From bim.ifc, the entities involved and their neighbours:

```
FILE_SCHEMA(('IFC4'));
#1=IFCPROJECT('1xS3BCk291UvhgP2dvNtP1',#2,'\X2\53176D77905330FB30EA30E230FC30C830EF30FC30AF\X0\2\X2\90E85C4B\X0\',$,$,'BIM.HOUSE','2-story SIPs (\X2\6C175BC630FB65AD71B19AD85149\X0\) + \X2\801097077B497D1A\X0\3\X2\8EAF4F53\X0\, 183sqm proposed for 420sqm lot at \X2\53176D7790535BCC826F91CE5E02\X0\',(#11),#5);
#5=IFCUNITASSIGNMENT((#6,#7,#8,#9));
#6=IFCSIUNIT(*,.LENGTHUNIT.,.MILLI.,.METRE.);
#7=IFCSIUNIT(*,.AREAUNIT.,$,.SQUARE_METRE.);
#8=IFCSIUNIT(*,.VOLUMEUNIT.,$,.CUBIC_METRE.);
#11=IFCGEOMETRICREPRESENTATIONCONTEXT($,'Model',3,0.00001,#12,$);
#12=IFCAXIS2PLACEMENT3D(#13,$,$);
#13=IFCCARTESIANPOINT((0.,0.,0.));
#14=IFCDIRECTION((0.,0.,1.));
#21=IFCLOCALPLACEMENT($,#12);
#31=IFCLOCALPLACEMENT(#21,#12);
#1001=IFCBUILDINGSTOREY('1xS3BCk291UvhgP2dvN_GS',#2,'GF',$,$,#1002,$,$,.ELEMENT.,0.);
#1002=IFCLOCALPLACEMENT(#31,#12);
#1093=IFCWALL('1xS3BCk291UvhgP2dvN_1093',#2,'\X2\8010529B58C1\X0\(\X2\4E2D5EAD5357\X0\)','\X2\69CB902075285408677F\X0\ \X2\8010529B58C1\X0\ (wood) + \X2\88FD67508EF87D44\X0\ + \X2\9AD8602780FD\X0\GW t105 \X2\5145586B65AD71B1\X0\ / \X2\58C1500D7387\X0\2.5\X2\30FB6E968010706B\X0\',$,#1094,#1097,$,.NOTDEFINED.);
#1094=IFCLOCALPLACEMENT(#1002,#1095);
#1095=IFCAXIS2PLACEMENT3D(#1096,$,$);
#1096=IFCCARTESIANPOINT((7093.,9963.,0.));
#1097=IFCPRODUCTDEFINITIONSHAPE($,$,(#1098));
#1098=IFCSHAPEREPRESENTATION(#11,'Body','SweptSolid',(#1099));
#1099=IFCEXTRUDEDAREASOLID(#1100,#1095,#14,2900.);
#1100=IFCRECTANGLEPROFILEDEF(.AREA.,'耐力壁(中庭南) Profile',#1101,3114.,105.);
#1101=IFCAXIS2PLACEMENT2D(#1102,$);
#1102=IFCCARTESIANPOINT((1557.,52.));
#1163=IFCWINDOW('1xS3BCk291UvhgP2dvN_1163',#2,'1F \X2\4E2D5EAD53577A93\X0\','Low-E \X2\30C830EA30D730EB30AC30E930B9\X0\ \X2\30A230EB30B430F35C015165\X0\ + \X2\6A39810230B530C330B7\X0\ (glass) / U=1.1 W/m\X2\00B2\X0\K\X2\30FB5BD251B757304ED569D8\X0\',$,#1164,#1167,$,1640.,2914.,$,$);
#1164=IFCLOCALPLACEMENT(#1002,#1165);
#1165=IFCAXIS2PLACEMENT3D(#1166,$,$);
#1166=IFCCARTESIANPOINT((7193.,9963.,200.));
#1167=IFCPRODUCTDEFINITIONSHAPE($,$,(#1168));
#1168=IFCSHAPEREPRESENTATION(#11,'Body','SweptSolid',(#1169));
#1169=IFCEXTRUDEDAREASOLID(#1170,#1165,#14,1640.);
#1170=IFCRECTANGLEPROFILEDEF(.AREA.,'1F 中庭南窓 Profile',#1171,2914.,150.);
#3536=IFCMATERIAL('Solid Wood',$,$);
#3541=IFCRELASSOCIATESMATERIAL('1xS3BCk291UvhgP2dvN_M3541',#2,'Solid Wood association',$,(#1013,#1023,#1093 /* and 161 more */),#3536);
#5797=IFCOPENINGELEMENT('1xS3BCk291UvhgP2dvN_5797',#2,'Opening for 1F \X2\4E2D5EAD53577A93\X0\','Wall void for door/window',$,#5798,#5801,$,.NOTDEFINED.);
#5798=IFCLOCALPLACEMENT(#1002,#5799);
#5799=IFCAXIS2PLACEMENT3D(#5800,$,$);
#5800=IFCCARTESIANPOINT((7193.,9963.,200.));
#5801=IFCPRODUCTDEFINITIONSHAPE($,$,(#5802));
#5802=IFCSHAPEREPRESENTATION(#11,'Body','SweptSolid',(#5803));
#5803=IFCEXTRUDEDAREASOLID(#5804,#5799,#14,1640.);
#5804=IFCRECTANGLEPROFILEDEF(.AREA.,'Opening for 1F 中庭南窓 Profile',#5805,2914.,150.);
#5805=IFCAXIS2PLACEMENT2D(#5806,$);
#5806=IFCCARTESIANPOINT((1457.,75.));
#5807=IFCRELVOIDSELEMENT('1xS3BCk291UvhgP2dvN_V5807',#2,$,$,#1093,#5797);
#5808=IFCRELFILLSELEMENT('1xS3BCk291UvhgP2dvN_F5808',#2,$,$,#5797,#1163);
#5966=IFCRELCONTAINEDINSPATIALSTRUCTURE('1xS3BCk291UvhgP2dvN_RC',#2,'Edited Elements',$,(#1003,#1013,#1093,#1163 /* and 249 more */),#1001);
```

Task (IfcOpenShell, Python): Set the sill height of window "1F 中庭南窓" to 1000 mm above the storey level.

```python
import numpy as np
import ifcopenshell
import ifcopenshell.api.geometry
import ifcopenshell.geom
import ifcopenshell.util.element
import ifcopenshell.util.placement
import ifcopenshell.util.shape
import ifcopenshell.util.unit

model = ifcopenshell.open("bim.ifc")
unit_scale = ifcopenshell.util.unit.calculate_unit_scale(model)

window = model.by_id(1163)
opening = window.FillsVoids[0].RelatingOpeningElement
storey = ifcopenshell.util.element.get_container(window, ifc_class="IfcBuildingStorey")
level = ifcopenshell.util.placement.get_local_placement(storey.ObjectPlacement)[2, 3]

# The opening's origin need not be at the sill, so measure its lowest point.
shape = ifcopenshell.geom.create_shape(ifcopenshell.geom.settings(), opening)
bottom = ifcopenshell.util.shape.get_shape_bottom_elevation(shape, shape.geometry) / unit_scale
dz = level + 1 / unit_scale - bottom

shift = np.array([0.0, 0.0, dz])
# The window is not placed relative to its opening, so move both.
for product in (opening, window):
    matrix = ifcopenshell.util.placement.get_local_placement(product.ObjectPlacement)
    matrix[:3, 3] += shift
    ifcopenshell.api.geometry.edit_object_placement(model, product=product, matrix=matrix, is_si=False)

print(f"moved by {dz * unit_scale:+.3f} m")

model.write("bim_v2.ifc")
```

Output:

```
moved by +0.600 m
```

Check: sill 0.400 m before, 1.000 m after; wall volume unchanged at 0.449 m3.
